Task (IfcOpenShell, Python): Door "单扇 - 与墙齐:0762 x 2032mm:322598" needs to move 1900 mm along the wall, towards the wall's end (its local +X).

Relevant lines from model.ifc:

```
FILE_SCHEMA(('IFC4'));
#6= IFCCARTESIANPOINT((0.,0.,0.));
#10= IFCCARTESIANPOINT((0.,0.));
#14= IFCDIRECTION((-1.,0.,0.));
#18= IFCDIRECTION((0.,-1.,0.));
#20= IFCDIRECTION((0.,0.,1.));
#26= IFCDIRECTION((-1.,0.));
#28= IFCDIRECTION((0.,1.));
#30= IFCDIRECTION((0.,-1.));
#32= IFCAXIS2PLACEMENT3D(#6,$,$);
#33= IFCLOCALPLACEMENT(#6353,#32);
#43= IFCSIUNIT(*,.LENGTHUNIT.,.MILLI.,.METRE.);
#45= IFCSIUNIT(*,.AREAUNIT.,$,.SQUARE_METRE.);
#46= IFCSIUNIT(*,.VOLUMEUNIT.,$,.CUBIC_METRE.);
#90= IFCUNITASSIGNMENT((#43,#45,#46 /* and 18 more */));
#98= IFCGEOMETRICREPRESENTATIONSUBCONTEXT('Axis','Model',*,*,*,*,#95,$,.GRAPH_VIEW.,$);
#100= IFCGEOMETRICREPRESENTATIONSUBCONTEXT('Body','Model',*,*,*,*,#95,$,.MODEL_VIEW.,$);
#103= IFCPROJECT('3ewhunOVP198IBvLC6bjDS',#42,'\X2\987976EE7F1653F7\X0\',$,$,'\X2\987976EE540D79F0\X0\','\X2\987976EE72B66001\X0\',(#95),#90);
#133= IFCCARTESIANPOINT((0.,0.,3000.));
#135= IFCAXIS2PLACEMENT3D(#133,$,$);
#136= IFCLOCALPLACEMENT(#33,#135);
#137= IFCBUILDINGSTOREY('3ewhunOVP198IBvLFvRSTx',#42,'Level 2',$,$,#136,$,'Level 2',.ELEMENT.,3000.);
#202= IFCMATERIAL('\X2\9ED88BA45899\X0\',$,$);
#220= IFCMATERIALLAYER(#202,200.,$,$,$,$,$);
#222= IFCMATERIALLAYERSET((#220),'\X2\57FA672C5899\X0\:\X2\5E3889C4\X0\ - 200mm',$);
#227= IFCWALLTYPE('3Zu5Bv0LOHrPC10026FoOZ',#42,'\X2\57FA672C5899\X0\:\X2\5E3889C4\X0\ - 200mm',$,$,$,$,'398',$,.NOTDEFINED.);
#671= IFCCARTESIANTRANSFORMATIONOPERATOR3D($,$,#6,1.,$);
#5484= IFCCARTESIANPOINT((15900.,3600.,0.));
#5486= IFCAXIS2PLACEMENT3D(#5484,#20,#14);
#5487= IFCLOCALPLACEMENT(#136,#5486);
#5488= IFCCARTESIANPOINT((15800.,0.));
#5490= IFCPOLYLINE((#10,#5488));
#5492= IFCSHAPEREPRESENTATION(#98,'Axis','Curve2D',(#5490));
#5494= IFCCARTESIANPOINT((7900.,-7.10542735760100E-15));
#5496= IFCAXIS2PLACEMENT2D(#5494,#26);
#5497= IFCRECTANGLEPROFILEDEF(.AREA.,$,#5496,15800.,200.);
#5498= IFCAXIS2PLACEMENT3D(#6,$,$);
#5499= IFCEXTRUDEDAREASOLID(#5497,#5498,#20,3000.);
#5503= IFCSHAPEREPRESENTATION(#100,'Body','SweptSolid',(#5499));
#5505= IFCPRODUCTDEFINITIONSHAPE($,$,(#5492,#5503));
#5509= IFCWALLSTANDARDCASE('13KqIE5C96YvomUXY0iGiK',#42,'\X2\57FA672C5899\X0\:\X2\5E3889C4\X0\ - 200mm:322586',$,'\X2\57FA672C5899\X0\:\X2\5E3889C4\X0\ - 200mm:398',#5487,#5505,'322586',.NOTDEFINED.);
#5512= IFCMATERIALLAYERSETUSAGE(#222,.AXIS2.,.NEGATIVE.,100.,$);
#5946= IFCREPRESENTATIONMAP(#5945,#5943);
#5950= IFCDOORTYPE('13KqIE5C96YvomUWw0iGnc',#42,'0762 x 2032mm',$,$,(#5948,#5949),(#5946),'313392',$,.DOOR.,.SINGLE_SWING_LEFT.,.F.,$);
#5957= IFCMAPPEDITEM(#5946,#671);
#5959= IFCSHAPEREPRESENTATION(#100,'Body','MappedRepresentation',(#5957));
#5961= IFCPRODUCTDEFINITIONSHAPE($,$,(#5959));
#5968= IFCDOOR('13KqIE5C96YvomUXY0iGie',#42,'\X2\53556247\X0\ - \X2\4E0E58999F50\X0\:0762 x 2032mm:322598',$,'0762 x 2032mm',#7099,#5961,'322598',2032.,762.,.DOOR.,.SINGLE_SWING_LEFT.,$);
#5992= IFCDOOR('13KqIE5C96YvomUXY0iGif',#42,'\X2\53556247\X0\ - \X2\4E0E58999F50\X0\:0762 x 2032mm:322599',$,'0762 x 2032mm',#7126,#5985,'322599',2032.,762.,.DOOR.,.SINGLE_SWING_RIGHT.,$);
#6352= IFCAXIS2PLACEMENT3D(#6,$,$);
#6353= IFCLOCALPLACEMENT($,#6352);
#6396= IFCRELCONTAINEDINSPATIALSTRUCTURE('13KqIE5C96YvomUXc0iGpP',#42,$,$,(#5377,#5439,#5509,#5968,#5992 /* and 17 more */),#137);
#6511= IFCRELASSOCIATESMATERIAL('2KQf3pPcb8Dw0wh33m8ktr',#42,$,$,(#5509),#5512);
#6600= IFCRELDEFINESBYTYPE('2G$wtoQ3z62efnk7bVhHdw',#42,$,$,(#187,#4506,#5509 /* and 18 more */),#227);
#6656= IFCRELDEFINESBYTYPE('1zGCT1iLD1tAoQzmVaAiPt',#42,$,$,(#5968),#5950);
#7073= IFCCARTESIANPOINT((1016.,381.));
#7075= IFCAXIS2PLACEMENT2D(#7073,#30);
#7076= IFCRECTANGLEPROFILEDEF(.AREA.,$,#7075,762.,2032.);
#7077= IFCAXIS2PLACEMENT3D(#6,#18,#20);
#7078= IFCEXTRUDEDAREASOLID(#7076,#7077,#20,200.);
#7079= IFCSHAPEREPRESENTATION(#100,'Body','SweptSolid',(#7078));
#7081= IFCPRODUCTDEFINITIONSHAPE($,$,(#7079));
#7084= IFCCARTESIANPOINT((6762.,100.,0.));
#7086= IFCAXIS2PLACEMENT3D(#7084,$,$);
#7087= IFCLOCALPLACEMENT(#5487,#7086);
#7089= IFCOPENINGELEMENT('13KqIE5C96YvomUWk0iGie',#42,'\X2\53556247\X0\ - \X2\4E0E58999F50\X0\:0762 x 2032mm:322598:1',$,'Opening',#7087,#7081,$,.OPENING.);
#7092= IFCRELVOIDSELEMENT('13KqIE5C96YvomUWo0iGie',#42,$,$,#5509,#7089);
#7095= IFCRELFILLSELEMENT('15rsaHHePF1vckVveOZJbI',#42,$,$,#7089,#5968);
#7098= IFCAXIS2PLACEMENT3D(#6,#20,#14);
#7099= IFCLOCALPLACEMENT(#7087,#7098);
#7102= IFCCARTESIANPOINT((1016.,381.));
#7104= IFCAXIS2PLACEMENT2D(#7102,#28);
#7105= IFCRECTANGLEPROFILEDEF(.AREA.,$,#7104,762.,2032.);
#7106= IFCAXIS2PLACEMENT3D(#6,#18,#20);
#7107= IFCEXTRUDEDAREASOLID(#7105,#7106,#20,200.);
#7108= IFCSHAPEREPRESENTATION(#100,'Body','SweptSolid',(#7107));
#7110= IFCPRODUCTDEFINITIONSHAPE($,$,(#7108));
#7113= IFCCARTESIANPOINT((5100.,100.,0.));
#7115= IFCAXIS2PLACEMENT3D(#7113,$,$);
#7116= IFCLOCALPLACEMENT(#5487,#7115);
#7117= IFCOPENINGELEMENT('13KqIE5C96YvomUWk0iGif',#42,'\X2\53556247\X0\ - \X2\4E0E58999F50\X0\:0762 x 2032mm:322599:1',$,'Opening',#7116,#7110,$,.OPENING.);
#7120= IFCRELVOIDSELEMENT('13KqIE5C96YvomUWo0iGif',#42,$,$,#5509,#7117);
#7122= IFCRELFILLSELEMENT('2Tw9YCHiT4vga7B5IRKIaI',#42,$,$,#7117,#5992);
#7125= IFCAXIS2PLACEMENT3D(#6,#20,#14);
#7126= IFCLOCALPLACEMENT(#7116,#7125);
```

```python
import ifcopenshell
import ifcopenshell.api.geometry
import ifcopenshell.util.placement
import ifcopenshell.util.unit

model = ifcopenshell.open("model.ifc")
unit_scale = ifcopenshell.util.unit.calculate_unit_scale(model)

door = model.by_guid("13KqIE5C96YvomUXY0iGie")
opening = door.FillsVoids[0].RelatingOpeningElement
wall = opening.VoidsElements[0].RelatingBuildingElement

wall_matrix = ifcopenshell.util.placement.get_local_placement(wall.ObjectPlacement)
shift = wall_matrix[:3, 0] * 1.9 / unit_scale
before = ifcopenshell.util.placement.get_local_placement(door.ObjectPlacement)[:3, 3].copy()

# The door is placed relative to its opening, so it follows when the opening moves.
matrix = ifcopenshell.util.placement.get_local_placement(opening.ObjectPlacement)
matrix[:3, 3] += shift
ifcopenshell.api.geometry.edit_object_placement(
    model, product=opening, matrix=matrix, is_si=False, should_transform_children=True
)

after = ifcopenshell.util.placement.get_local_placement(door.ObjectPlacement)[:3, 3]
print("door moved by", (after - before).round(3) + 0.0)

model.write("model_v2.ifc")
```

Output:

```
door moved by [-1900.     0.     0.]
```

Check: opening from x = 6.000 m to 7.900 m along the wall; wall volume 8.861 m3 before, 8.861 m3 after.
